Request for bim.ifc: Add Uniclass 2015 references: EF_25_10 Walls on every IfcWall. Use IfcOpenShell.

First a look at what the model holds.

```python
import ifcopenshell

model = ifcopenshell.open("bim.ifc")
print(model.schema)
print("classifications:", [c.Name for c in model.by_type("IfcClassification")])
for ifc_class in ("IfcDoor", "IfcRoof", "IfcStair", "IfcWall", "IfcWindow"):
    print(ifc_class, len(model.by_type(ifc_class)))
```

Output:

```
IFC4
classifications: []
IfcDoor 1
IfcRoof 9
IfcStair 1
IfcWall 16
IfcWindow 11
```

```python
import ifcopenshell
import ifcopenshell.api.classification

model = ifcopenshell.open("bim.ifc")

system = ifcopenshell.api.classification.add_classification(model, classification="Uniclass 2015")

codes = {
    "IfcWall": ("EF_25_10", "Walls"),
}
for ifc_class, (code, name) in codes.items():
    products = model.by_type(ifc_class)
    ifcopenshell.api.classification.add_reference(
        model, products=products, classification=system, identification=code, name=name
    )
    print(code, len(products))

model.write("bim_updated.ifc")
```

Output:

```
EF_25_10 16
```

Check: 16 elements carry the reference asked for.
